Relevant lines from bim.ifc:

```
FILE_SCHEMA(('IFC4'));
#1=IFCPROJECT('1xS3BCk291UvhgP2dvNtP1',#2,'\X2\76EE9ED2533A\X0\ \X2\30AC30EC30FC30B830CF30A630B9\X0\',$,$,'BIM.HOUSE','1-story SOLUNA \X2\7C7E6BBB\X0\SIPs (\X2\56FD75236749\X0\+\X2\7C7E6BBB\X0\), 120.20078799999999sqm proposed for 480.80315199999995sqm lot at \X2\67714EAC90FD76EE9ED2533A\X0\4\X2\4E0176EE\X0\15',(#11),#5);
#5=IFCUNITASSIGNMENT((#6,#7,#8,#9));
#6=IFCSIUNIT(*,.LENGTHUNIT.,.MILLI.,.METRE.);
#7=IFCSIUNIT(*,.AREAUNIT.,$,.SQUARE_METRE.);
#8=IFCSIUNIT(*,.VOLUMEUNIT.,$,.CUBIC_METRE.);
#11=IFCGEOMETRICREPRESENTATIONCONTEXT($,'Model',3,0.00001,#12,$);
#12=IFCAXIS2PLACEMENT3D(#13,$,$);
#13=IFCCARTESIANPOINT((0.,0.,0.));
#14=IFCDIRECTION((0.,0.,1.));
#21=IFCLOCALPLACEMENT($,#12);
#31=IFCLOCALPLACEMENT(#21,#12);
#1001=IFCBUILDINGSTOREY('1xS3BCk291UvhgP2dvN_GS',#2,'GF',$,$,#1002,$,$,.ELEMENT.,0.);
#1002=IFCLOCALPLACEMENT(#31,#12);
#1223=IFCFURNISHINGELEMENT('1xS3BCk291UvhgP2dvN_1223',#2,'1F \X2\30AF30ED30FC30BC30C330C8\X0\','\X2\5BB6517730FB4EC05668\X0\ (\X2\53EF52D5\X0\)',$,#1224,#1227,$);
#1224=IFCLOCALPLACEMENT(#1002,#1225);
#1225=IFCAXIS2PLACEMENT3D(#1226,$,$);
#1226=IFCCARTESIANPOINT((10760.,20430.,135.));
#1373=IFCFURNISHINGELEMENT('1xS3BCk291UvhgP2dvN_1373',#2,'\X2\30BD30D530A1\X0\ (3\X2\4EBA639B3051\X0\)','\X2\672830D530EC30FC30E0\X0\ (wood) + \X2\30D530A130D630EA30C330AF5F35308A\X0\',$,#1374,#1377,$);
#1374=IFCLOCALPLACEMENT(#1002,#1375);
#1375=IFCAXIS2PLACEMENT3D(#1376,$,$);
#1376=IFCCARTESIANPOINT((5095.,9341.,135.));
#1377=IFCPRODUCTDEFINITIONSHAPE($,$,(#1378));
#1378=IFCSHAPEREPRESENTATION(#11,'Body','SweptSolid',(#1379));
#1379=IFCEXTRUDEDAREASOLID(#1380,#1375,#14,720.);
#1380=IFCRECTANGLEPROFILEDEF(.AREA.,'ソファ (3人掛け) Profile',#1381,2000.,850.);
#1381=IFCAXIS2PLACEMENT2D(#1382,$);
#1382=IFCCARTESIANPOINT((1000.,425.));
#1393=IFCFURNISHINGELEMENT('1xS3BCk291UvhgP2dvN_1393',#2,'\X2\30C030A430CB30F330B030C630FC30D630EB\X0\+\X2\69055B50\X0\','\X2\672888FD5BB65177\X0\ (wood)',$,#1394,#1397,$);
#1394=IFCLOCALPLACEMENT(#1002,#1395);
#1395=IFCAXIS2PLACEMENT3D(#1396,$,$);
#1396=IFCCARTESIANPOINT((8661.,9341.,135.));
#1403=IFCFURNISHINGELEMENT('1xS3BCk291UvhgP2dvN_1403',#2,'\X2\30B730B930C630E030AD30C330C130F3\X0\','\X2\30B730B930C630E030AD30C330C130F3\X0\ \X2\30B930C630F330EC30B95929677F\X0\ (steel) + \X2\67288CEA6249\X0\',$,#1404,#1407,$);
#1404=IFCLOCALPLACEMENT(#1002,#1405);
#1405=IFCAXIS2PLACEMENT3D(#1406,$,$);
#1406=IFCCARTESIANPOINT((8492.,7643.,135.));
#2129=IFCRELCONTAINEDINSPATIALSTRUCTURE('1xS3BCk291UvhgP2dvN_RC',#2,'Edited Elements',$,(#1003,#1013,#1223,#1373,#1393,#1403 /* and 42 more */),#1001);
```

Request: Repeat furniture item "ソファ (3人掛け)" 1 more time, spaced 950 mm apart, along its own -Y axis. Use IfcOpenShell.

```python
import ifcopenshell
import ifcopenshell.api.geometry
import ifcopenshell.api.root
import ifcopenshell.util.element
import ifcopenshell.util.placement
import ifcopenshell.util.unit

model = ifcopenshell.open("bim.ifc")
unit_scale = ifcopenshell.util.unit.calculate_unit_scale(model)


def reuse_history(source, copy):
    """copy_class also copies each property set's owner history, people and application; keep the originals."""
    for rel in copy.IsDefinedBy:
        if rel.is_a("IfcRelDefinesByProperties") and (history := rel.RelatingPropertyDefinition.OwnerHistory):
            rel.RelatingPropertyDefinition.OwnerHistory = source.OwnerHistory
            ifcopenshell.util.element.remove_deep2(model, history)


source = model.by_id(1373)
base = ifcopenshell.util.placement.get_local_placement(source.ObjectPlacement)
step = -base[:3, 1] * 0.95 / unit_scale

for i in range(1, 2):
    copy = ifcopenshell.api.root.copy_class(model, product=source)
    copy.Representation = ifcopenshell.util.element.copy_deep(
        model, source.Representation, exclude=["IfcGeometricRepresentationContext", "IfcRepresentationMap"]
    )
    reuse_history(source, copy)
    matrix = base.copy()
    matrix[:3, 3] += i * step
    print("added at", matrix[:3, 3].round(3) + 0.0)
    ifcopenshell.api.geometry.edit_object_placement(model, product=copy, matrix=matrix, is_si=False)

model.write("bim_rev.ifc")
```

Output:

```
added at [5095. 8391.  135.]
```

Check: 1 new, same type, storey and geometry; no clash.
